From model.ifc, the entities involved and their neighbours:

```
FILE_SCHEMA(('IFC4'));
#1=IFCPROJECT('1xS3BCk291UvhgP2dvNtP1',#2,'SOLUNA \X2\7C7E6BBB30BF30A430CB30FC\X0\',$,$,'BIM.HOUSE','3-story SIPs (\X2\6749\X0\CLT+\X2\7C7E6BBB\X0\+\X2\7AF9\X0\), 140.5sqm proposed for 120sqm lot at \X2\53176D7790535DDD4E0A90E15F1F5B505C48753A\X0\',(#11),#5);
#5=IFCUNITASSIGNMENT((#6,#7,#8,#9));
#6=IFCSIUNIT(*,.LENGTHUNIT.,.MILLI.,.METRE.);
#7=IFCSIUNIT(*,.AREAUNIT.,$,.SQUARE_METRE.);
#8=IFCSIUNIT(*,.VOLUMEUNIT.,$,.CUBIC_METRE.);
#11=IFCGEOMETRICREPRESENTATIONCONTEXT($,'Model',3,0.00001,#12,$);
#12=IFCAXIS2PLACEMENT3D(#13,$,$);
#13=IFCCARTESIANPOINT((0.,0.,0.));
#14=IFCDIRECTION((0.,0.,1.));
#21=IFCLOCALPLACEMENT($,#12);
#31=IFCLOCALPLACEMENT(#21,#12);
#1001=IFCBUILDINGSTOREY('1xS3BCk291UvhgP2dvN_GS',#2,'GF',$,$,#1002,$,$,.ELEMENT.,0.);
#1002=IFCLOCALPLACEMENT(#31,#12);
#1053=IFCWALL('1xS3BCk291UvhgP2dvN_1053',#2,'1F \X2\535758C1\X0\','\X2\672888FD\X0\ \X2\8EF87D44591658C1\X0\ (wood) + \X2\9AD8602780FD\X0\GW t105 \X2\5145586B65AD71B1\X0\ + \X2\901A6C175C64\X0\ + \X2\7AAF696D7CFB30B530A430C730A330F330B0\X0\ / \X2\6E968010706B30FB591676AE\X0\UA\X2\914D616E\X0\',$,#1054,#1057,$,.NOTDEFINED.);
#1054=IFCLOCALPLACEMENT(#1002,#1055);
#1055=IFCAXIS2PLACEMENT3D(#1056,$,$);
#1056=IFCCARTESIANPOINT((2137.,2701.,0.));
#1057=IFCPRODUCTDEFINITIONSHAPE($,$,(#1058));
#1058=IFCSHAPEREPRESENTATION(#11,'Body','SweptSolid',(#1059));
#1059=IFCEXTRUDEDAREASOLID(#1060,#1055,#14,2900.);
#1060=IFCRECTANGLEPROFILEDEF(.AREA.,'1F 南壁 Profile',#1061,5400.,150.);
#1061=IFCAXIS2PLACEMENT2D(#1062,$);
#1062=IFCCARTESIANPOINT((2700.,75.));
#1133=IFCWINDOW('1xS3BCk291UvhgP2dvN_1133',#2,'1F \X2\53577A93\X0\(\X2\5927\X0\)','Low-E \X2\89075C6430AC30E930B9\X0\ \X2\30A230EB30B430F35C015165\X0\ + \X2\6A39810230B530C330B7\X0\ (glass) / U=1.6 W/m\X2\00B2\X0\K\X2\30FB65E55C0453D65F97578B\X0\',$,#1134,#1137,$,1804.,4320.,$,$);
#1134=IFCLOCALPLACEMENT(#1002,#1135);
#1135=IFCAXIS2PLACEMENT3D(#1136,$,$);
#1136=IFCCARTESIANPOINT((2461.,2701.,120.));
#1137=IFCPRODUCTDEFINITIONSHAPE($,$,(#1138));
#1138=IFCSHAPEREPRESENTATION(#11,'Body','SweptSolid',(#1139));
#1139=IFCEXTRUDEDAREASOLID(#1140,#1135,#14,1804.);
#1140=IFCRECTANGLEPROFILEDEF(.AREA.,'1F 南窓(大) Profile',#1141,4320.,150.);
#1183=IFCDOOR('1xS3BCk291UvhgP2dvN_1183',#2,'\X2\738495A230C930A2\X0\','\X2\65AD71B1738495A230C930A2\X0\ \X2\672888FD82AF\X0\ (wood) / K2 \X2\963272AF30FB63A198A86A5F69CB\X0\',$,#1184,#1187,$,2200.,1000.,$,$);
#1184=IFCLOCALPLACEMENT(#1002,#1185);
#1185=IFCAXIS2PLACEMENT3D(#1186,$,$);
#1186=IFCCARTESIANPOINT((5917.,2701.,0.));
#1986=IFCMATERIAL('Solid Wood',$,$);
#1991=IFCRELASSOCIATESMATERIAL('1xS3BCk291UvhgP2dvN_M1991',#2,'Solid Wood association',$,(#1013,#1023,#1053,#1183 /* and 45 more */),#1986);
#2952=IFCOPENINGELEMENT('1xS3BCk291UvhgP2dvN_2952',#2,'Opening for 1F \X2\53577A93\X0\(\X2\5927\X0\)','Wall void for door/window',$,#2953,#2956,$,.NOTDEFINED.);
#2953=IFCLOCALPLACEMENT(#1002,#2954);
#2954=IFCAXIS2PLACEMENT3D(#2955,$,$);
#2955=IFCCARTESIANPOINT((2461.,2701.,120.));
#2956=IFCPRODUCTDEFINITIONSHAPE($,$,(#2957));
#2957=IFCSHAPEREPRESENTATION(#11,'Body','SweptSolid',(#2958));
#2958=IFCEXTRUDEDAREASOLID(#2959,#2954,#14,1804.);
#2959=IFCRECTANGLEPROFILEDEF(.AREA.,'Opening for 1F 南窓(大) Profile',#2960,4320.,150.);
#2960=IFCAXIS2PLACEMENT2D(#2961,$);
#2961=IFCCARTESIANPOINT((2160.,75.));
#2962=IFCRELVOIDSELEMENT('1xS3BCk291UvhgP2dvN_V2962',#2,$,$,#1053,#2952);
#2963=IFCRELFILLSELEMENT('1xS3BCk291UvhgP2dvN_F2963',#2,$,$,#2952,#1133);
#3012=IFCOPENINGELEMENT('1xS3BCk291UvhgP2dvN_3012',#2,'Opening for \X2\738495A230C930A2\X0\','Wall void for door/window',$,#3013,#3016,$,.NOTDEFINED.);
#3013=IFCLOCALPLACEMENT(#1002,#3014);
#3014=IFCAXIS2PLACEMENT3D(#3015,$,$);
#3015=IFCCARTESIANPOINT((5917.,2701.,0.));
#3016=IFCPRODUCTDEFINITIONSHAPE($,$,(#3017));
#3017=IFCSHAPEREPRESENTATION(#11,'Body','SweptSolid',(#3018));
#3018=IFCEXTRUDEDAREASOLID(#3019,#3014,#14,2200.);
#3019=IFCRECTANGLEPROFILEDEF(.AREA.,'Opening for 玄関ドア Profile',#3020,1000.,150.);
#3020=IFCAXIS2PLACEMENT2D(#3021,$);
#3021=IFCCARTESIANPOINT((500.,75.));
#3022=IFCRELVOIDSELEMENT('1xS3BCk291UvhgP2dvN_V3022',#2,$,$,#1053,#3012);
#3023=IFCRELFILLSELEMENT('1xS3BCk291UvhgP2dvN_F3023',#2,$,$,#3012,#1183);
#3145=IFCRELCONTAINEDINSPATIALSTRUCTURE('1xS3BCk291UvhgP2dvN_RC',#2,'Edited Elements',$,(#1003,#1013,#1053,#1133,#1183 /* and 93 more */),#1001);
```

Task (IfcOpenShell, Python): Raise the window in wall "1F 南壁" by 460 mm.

```python
import numpy as np
import ifcopenshell
import ifcopenshell.api.geometry
import ifcopenshell.util.placement
import ifcopenshell.util.unit

model = ifcopenshell.open("model.ifc")
unit_scale = ifcopenshell.util.unit.calculate_unit_scale(model)

window = model.by_id(1133)
opening = window.FillsVoids[0].RelatingOpeningElement
dz = 460.0

shift = np.array([0.0, 0.0, dz])
# The window is not placed relative to its opening, so move both.
for product in (opening, window):
    matrix = ifcopenshell.util.placement.get_local_placement(product.ObjectPlacement)
    matrix[:3, 3] += shift
    ifcopenshell.api.geometry.edit_object_placement(model, product=product, matrix=matrix, is_si=False)

print(f"moved by {dz * unit_scale:+.3f} m")

model.write("model_updated.ifc")
```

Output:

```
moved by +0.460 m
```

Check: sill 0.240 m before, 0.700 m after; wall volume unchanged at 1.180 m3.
